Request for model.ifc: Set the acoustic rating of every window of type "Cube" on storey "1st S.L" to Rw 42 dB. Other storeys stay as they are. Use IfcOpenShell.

First a look at what the model holds.

```python
import ifcopenshell
import ifcopenshell.util.element

model = ifcopenshell.open("model.ifc")
print(model.schema)
storey = next(s for s in model.by_type("IfcBuildingStorey") if s.Name == "1st S.L")
windows = [e for e in ifcopenshell.util.element.get_decomposition(storey) if e.is_a("IfcWindow")]
seen = {}
for e in windows:
    element_type = ifcopenshell.util.element.get_type(e)
    key = (element_type.Name if element_type != e and element_type else None, ifcopenshell.util.element.get_pset(e, "Pset_WindowCommon", "AcousticRating"))
    seen[key] = seen.get(key, 0) + 1
for (name, value), count in sorted(seen.items(), key=str):
    print(count, "x", name, "|", value)
```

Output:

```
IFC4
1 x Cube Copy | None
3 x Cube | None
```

```python
import ifcopenshell
import ifcopenshell.api.pset
import ifcopenshell.util.element

model = ifcopenshell.open("model.ifc")

storey = next(s for s in model.by_type("IfcBuildingStorey") if s.Name == "1st S.L")
windows = [e for e in ifcopenshell.util.element.get_decomposition(storey) if e.is_a("IfcWindow")]

count = 0
for e in windows:
    element_type = ifcopenshell.util.element.get_type(e)
    if element_type in (None, e) or element_type.Name != "Cube":
        continue
    # add_pset returns the element's existing set when there is one.
    pset = ifcopenshell.api.pset.add_pset(model, product=e, name="Pset_WindowCommon")
    ifcopenshell.api.pset.edit_pset(model, pset=pset, properties={"AcousticRating": "Rw 42 dB"})
    count += 1

print(count, "windows updated")

model.write("model_edited.ifc")
```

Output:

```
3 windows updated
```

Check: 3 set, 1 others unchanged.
